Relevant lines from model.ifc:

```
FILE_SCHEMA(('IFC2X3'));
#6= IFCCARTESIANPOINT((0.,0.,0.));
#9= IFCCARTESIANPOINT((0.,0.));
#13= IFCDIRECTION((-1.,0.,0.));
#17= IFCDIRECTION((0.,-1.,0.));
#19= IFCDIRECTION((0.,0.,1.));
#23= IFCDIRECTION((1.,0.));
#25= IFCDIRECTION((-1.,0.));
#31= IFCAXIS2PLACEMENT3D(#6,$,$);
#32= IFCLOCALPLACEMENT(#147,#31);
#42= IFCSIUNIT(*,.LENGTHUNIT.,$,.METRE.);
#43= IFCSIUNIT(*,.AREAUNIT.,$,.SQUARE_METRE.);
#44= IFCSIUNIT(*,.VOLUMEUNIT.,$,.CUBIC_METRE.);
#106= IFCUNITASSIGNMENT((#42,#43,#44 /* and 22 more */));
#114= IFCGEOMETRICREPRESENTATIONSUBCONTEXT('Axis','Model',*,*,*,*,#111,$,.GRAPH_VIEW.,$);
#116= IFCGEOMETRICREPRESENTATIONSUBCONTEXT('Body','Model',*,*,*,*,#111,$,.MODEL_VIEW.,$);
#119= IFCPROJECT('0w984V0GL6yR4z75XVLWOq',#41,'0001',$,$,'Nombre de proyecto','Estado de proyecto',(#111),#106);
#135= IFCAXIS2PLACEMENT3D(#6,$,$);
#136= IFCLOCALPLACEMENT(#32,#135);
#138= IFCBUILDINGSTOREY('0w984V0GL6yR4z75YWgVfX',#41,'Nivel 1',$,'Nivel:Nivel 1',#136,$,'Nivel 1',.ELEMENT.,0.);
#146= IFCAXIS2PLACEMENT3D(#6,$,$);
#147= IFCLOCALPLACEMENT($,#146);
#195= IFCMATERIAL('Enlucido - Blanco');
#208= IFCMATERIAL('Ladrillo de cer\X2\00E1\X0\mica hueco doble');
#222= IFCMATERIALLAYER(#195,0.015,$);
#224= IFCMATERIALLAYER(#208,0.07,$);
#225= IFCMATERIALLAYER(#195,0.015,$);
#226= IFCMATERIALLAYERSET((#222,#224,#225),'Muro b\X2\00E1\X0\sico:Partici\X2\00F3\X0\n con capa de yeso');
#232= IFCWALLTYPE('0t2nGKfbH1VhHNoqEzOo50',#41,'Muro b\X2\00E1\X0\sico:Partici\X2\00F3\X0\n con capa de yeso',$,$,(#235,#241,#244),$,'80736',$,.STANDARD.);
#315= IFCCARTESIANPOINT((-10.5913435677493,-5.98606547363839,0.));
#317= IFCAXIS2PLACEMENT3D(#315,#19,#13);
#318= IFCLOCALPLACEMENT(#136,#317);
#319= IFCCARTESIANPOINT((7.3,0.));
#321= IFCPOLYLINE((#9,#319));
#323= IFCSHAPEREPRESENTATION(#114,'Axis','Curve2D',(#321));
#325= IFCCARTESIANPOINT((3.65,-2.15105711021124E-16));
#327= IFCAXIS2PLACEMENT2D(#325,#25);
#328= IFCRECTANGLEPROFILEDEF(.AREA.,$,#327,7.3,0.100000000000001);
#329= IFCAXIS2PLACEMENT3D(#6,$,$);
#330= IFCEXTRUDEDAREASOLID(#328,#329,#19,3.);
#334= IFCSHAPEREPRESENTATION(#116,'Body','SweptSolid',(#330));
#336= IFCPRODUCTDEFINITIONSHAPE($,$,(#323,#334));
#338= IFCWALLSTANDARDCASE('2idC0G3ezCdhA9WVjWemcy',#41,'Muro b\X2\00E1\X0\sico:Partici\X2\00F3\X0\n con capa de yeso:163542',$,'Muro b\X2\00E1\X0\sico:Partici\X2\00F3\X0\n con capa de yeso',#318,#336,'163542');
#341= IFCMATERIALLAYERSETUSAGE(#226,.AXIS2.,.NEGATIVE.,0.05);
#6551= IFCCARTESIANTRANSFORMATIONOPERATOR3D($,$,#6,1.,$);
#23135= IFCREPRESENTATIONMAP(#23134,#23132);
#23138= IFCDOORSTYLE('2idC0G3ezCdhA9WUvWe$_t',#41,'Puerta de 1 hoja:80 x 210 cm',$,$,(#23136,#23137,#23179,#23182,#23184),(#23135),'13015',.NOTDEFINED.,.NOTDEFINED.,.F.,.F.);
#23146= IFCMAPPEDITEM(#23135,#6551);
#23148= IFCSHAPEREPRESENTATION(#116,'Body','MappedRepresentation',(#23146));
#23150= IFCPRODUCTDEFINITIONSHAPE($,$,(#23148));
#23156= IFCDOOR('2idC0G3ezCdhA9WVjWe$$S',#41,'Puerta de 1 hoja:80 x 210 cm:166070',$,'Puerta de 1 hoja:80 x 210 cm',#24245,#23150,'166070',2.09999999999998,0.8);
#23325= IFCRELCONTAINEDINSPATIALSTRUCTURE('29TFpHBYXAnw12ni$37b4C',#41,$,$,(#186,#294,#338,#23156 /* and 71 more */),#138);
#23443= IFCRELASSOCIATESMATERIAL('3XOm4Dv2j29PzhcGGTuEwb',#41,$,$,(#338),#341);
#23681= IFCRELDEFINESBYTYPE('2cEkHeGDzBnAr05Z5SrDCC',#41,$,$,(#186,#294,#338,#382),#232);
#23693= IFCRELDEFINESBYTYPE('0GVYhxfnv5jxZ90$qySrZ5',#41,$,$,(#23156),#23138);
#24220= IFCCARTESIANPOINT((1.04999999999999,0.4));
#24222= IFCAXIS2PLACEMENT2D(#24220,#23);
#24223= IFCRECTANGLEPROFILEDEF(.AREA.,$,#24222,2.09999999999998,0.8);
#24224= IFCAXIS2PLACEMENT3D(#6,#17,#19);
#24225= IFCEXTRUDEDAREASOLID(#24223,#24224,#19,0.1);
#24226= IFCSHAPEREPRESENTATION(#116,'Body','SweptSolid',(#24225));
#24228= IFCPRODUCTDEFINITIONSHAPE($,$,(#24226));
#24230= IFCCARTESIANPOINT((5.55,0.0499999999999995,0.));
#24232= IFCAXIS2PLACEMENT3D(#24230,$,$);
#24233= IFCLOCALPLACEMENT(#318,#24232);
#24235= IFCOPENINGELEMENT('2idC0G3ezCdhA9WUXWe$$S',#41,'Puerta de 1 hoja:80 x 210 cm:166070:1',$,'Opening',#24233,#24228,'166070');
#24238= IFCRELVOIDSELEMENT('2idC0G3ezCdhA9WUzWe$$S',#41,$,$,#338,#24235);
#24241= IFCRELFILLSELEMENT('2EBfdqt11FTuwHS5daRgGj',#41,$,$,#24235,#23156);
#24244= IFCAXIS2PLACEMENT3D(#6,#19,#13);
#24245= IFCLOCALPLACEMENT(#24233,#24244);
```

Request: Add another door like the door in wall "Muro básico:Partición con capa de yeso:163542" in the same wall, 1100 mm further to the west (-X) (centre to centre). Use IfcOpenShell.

```python
import ifcopenshell
import ifcopenshell.api.feature
import ifcopenshell.api.geometry
import ifcopenshell.api.root
import ifcopenshell.geom
import ifcopenshell.util.element
import ifcopenshell.util.placement
import ifcopenshell.util.shape
import ifcopenshell.util.unit

model = ifcopenshell.open("model.ifc")
unit_scale = ifcopenshell.util.unit.calculate_unit_scale(model)
settings = ifcopenshell.geom.settings()


def volume(element):
    """Net volume in cubic metres, openings subtracted."""
    shape = ifcopenshell.geom.create_shape(settings, element)
    return ifcopenshell.util.shape.get_volume(shape.geometry)


def reuse_history(source, copy):
    """copy_class also copies each property set's owner history, people and application; keep the originals."""
    for rel in copy.IsDefinedBy:
        if rel.is_a("IfcRelDefinesByProperties") and (history := rel.RelatingPropertyDefinition.OwnerHistory):
            rel.RelatingPropertyDefinition.OwnerHistory = source.OwnerHistory
            ifcopenshell.util.element.remove_deep2(model, history)


door = model.by_id(23156)
opening = door.FillsVoids[0].RelatingOpeningElement
wall = opening.VoidsElements[0].RelatingBuildingElement
before = volume(wall)
shift = ifcopenshell.util.placement.get_local_placement(wall.ObjectPlacement)[:3, 0] * 1.1 / unit_scale

# copy_class copies the void relationship, type, container and properties, but no geometry.
new_opening = ifcopenshell.api.root.copy_class(model, product=opening)
new_opening.Representation = ifcopenshell.util.element.copy_deep(
    model, opening.Representation, exclude=["IfcGeometricRepresentationContext", "IfcRepresentationMap"]
)
new_opening.Name = "Puerta de 1 hoja:80 x 210 cm"
new_opening.Tag = None
new_door = ifcopenshell.api.root.copy_class(model, product=door)
new_door.Representation = ifcopenshell.util.element.copy_deep(
    model, door.Representation, exclude=["IfcGeometricRepresentationContext", "IfcRepresentationMap"]
)
new_door.Name = "Puerta de 1 hoja:80 x 210 cm"
new_door.Tag = None
reuse_history(door, new_door)
fills = ifcopenshell.api.feature.add_filling(model, opening=new_opening, element=new_door)
fills.OwnerHistory = new_door.OwnerHistory  # required in IFC2X3

for old, new in ((opening, new_opening), (door, new_door)):
    matrix = ifcopenshell.util.placement.get_local_placement(old.ObjectPlacement)
    matrix[:3, 3] += shift
    ifcopenshell.api.geometry.edit_object_placement(model, product=new, matrix=matrix, is_si=False)

after = volume(wall)

print(f"wall volume {before:.3f} -> {after:.3f} m3")

model.write("model_edited.ifc")
```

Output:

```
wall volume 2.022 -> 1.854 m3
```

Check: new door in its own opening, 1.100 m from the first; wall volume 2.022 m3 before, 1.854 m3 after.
